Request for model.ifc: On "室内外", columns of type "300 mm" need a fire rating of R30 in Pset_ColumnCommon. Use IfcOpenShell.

First a look at what the model holds.

```python
import ifcopenshell
import ifcopenshell.util.element

model = ifcopenshell.open("model.ifc")
print(model.schema)
storey = next(s for s in model.by_type("IfcBuildingStorey") if s.Name == "室内外")
columns = [e for e in ifcopenshell.util.element.get_decomposition(storey) if e.is_a("IfcColumn")]
seen = {}
for e in columns:
    element_type = ifcopenshell.util.element.get_type(e)
    key = (element_type.Name if element_type != e and element_type else None, ifcopenshell.util.element.get_pset(e, "Pset_ColumnCommon", "FireRating"))
    seen[key] = seen.get(key, 0) + 1
for (name, value), count in sorted(seen.items(), key=str):
    print(count, "x", name, "|", value)
```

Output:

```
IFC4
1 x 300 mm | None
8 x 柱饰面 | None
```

```python
import ifcopenshell
import ifcopenshell.api.pset
import ifcopenshell.util.element

model = ifcopenshell.open("model.ifc")

storey = next(s for s in model.by_type("IfcBuildingStorey") if s.Name == "室内外")
columns = [e for e in ifcopenshell.util.element.get_decomposition(storey) if e.is_a("IfcColumn")]

count = 0
for e in columns:
    element_type = ifcopenshell.util.element.get_type(e)
    if element_type in (None, e) or element_type.Name != "300 mm":
        continue
    # add_pset returns the element's existing set when there is one.
    pset = ifcopenshell.api.pset.add_pset(model, product=e, name="Pset_ColumnCommon")
    ifcopenshell.api.pset.edit_pset(model, pset=pset, properties={"FireRating": "R30"})
    count += 1

print(count, "columns updated")

model.write("model_updated.ifc")
```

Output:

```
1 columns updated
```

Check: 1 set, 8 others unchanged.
